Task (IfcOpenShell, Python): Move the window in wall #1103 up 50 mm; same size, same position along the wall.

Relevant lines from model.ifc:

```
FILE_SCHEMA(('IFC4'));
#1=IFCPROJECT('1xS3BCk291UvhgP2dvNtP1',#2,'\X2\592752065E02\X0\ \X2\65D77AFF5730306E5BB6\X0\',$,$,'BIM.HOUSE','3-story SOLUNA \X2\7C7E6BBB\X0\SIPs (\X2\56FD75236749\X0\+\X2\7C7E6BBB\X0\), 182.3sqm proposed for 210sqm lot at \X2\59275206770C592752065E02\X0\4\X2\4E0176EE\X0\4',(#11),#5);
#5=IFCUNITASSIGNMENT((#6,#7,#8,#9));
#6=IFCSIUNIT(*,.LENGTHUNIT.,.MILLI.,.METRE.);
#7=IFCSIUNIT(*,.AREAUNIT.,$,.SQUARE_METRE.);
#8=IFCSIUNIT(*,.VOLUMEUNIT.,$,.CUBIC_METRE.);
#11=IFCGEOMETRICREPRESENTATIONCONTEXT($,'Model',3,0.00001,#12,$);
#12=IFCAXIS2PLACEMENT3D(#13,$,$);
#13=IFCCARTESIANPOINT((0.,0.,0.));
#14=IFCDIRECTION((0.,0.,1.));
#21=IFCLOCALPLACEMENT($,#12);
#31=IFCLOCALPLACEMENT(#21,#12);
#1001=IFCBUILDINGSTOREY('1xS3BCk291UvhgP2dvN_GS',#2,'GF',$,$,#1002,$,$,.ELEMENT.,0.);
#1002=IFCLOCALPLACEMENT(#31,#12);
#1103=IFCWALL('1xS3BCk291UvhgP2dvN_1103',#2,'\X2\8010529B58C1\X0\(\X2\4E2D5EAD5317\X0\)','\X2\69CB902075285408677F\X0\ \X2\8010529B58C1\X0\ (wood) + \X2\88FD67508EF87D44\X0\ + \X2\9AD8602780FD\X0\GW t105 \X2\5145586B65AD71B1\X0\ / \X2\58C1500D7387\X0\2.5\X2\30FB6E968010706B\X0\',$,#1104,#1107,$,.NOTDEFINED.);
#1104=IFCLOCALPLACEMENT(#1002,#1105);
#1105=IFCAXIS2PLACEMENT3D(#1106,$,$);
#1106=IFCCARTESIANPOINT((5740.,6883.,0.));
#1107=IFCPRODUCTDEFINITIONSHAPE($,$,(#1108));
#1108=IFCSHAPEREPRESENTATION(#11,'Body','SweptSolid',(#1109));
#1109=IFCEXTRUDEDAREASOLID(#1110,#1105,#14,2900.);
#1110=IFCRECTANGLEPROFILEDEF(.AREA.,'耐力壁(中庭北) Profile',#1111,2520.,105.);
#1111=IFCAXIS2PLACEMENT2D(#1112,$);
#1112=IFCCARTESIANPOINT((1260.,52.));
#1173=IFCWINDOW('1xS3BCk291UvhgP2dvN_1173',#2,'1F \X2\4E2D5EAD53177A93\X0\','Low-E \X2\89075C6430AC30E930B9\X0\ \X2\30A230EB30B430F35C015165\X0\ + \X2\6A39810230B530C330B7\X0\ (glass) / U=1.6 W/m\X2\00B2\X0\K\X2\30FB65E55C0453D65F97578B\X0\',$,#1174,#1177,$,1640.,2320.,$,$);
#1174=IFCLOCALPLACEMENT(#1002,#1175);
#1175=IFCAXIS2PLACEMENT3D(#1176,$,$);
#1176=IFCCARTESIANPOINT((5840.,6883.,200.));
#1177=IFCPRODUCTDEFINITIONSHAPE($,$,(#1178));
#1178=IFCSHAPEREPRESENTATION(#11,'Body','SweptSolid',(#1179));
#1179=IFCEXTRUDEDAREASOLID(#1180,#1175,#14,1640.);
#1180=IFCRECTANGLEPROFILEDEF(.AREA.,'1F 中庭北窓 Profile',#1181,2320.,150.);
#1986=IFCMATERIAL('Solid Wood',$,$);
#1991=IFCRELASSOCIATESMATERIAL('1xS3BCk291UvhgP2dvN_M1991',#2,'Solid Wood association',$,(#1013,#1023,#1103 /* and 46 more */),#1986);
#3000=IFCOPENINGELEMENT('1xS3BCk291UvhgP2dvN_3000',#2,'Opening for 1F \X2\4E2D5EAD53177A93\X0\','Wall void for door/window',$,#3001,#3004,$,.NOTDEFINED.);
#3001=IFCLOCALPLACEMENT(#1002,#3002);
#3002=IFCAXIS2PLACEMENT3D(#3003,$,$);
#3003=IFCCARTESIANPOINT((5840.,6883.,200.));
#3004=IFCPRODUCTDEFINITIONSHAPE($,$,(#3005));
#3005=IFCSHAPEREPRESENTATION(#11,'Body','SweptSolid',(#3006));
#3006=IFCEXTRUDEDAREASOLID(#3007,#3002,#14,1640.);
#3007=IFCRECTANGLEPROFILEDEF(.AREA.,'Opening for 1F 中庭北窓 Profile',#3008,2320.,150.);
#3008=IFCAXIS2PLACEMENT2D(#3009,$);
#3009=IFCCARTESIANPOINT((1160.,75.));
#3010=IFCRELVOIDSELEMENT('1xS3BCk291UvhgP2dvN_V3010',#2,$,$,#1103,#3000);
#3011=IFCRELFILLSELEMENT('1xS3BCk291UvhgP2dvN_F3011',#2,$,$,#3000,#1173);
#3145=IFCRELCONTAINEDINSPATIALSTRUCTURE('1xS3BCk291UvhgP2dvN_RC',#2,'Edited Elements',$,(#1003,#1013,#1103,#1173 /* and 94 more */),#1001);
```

```python
import numpy as np
import ifcopenshell
import ifcopenshell.api.geometry
import ifcopenshell.util.placement
import ifcopenshell.util.unit

model = ifcopenshell.open("model.ifc")
unit_scale = ifcopenshell.util.unit.calculate_unit_scale(model)

window = model.by_guid("1xS3BCk291UvhgP2dvN_1173")
opening = window.FillsVoids[0].RelatingOpeningElement
dz = 0.05 / unit_scale

shift = np.array([0.0, 0.0, dz])
# The window is not placed relative to its opening, so move both.
for product in (opening, window):
    matrix = ifcopenshell.util.placement.get_local_placement(product.ObjectPlacement)
    matrix[:3, 3] += shift
    ifcopenshell.api.geometry.edit_object_placement(model, product=product, matrix=matrix, is_si=False)

print(f"moved by {dz * unit_scale:+.3f} m")

model.write("model_updated.ifc")
```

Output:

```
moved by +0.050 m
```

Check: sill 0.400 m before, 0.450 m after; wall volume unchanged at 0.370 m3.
